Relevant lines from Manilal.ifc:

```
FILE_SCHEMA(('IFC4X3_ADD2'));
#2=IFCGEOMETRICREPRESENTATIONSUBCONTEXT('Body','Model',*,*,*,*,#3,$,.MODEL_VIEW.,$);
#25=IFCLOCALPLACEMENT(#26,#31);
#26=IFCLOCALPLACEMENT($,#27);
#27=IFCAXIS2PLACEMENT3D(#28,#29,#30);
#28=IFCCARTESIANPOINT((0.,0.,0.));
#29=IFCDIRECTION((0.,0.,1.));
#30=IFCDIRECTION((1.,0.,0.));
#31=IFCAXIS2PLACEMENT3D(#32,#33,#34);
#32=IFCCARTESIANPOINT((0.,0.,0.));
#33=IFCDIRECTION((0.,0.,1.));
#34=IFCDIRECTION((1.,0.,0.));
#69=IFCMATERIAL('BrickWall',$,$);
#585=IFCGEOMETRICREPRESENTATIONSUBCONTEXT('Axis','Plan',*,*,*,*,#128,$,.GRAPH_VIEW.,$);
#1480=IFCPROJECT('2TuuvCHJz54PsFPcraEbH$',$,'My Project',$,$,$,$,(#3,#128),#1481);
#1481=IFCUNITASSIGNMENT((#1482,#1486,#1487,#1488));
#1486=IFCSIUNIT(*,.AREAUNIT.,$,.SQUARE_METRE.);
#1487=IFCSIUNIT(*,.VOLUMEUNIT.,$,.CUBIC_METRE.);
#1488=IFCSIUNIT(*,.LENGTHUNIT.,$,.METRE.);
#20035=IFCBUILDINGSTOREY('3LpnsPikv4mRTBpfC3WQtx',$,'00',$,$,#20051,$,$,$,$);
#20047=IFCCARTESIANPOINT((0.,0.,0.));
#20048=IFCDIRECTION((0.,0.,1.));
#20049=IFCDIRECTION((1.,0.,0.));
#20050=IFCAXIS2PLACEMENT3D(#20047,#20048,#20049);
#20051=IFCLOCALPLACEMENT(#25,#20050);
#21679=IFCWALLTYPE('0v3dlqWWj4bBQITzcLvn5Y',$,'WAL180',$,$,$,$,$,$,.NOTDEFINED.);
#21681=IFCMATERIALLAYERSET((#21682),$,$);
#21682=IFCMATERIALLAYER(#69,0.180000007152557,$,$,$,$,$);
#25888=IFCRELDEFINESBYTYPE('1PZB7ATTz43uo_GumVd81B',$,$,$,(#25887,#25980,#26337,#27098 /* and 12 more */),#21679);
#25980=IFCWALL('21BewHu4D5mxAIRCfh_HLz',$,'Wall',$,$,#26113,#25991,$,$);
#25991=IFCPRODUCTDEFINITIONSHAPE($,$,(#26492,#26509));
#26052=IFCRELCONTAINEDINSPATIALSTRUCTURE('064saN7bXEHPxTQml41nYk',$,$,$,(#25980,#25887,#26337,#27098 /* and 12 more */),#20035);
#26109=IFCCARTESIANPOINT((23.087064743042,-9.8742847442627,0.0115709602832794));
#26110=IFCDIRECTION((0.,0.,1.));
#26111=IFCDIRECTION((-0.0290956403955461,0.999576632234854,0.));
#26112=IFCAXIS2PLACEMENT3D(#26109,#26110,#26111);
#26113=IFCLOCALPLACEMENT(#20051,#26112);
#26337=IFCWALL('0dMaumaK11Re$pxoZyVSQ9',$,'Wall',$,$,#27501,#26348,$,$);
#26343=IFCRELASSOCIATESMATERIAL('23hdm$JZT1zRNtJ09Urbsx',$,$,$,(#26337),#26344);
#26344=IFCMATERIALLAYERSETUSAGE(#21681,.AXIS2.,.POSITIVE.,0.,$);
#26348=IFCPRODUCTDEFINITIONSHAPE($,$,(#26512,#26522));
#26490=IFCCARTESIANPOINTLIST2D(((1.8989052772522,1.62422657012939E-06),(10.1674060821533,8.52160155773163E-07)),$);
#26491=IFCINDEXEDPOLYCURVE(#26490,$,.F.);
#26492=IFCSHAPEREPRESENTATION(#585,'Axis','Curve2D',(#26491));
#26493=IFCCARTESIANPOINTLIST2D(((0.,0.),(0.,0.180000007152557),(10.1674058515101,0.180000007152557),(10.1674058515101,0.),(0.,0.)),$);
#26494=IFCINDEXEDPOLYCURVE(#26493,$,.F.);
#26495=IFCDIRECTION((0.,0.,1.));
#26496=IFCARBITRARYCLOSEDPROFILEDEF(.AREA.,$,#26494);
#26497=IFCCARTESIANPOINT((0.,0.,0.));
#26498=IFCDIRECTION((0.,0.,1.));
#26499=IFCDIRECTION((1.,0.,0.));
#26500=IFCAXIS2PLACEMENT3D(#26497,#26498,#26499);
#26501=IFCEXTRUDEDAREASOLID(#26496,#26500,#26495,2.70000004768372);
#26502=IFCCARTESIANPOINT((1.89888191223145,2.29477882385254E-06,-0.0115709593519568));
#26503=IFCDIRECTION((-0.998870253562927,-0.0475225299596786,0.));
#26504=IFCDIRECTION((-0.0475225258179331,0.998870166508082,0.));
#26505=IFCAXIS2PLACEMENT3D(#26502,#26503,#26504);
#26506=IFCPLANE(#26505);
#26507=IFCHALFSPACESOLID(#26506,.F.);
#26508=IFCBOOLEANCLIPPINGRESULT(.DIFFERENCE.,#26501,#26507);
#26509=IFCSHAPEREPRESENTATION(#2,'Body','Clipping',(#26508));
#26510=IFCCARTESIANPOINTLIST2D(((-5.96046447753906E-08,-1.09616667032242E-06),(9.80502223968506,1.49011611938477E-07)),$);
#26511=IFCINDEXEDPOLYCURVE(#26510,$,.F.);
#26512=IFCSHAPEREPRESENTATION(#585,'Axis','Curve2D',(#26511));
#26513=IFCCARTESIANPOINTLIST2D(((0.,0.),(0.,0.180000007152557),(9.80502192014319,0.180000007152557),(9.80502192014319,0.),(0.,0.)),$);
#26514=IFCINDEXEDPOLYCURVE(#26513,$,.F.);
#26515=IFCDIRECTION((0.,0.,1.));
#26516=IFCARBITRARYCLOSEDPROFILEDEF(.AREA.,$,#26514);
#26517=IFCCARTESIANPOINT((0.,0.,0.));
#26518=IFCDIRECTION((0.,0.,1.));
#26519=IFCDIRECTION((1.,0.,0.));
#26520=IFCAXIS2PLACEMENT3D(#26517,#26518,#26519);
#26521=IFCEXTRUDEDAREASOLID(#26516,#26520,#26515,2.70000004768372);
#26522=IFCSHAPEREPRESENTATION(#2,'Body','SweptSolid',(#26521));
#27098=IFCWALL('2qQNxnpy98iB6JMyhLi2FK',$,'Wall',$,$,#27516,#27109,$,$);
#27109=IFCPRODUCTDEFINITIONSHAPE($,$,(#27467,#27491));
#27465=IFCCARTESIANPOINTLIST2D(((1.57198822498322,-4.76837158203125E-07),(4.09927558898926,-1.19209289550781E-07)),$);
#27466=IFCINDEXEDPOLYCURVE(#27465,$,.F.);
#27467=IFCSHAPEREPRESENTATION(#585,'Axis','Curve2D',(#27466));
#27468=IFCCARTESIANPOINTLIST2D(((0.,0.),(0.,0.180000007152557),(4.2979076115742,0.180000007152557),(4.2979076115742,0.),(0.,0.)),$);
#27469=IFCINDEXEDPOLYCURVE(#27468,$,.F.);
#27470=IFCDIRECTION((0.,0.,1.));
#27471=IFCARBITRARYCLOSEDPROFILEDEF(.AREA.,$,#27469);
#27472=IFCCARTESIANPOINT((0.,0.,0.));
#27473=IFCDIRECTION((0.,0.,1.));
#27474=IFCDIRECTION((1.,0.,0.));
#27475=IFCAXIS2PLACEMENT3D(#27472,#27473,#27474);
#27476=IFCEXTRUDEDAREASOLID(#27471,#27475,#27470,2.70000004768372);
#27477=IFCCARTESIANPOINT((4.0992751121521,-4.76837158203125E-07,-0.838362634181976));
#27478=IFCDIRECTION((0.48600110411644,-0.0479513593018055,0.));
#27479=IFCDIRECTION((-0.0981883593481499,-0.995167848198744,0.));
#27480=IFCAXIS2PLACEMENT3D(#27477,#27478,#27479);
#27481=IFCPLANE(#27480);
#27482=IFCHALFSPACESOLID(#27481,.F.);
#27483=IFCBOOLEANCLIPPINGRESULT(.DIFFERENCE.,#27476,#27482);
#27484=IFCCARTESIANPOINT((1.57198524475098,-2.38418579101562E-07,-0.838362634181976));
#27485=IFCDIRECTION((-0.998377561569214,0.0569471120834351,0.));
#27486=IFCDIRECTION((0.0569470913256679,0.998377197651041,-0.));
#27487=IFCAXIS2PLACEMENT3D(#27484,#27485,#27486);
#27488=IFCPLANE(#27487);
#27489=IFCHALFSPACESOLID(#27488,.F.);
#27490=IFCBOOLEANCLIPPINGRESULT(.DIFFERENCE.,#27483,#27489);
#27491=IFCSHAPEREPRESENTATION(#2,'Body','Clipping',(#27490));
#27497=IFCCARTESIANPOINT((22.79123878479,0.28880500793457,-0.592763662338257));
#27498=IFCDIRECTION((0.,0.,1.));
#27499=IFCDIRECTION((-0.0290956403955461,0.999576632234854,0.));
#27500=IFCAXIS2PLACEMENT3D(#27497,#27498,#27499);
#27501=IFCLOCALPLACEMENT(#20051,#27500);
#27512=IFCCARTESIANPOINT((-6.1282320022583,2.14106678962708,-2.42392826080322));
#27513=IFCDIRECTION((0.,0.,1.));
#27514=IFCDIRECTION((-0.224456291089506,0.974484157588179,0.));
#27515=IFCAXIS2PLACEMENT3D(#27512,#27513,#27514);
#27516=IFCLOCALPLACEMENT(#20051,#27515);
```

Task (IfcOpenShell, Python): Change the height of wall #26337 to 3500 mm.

```python
import ifcopenshell
import ifcopenshell.geom
import ifcopenshell.util.representation
import ifcopenshell.util.shape

model = ifcopenshell.open("Manilal.ifc")
settings = ifcopenshell.geom.settings()


def volume(element):
    """Net volume in cubic metres, openings subtracted."""
    shape = ifcopenshell.geom.create_shape(settings, element)
    return ifcopenshell.util.shape.get_volume(shape.geometry)


wall = model.by_guid("0dMaumaK11Re$pxoZyVSQ9")
before = volume(wall)

body = ifcopenshell.util.representation.get_representation(wall, "Model", "Body")
solid = body.Items[0]
old_height = solid.Depth
solid.Depth = 3.5
after = volume(wall)

print(f"height {old_height:g} -> {solid.Depth:g}, volume {before:.3f} -> {after:.3f} m3")

model.write("Manilal_edited.ifc")
```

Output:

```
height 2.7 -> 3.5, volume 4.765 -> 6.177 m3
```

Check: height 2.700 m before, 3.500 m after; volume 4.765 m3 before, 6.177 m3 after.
